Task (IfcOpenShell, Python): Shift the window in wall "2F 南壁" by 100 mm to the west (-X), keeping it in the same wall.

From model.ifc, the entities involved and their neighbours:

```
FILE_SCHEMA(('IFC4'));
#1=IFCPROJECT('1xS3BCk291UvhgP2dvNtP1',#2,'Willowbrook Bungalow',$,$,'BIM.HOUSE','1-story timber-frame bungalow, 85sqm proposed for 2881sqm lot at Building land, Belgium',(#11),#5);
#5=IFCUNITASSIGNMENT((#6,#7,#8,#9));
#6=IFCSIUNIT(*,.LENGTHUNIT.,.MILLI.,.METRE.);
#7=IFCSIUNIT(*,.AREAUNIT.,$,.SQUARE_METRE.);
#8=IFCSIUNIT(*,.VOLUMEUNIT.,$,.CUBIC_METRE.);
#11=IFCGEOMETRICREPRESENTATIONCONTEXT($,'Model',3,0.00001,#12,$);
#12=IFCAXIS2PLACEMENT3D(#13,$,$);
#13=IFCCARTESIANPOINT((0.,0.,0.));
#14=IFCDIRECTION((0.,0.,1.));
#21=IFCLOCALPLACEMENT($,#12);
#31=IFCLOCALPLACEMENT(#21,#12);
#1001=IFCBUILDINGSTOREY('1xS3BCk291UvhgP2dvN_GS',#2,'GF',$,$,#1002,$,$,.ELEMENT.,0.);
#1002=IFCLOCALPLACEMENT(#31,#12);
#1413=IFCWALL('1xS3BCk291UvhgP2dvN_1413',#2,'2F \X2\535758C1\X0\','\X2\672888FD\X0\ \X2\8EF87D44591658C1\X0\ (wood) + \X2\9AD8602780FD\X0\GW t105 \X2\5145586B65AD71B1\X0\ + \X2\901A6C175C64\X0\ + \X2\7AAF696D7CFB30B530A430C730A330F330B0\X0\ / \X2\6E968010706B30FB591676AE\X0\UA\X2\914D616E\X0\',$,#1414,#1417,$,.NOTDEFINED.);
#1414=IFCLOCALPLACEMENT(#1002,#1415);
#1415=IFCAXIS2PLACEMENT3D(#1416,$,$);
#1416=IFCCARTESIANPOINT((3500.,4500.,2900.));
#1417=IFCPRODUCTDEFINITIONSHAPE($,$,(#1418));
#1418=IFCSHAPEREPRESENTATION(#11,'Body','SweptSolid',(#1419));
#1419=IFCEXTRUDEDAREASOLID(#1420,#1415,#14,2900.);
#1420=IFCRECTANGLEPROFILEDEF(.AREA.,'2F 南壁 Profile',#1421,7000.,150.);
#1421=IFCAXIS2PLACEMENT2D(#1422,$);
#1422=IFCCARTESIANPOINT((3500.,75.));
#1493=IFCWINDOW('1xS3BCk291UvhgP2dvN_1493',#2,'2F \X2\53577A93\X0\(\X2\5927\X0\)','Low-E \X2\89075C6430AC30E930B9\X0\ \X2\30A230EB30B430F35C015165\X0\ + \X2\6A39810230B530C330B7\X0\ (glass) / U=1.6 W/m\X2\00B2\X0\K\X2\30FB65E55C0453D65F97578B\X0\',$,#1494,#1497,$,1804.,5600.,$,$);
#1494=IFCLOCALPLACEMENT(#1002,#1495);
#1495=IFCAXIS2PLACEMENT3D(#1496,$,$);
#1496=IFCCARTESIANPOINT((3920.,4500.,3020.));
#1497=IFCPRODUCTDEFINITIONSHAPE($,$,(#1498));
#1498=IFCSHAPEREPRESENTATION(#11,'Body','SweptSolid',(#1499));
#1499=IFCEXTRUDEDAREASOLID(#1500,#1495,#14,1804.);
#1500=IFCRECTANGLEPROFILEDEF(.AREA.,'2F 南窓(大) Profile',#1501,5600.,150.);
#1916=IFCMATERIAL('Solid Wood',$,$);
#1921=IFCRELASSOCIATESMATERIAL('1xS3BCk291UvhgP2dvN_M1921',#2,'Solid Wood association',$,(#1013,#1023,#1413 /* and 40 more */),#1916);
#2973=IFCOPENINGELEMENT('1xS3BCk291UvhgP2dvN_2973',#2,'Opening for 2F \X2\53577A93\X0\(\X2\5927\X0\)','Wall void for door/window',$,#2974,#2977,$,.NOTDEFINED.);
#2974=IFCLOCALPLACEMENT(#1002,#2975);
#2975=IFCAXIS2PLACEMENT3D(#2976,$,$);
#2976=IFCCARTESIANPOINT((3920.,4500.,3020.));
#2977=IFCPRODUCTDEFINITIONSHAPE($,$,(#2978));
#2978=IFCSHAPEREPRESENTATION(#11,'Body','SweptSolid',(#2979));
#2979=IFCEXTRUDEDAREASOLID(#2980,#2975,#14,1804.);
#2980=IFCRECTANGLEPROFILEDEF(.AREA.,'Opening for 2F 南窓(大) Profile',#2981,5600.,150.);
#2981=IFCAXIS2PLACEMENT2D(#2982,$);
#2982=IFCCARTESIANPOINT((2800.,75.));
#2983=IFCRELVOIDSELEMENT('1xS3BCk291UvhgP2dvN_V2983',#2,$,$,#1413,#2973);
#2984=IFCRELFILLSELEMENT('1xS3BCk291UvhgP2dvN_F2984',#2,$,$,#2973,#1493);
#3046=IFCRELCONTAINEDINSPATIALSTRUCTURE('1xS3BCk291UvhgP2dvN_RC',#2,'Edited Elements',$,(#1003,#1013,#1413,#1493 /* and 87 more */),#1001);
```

```python
import ifcopenshell
import ifcopenshell.api.geometry
import ifcopenshell.util.placement
import ifcopenshell.util.unit

model = ifcopenshell.open("model.ifc")
unit_scale = ifcopenshell.util.unit.calculate_unit_scale(model)

window = model.by_guid("1xS3BCk291UvhgP2dvN_1493")
opening = window.FillsVoids[0].RelatingOpeningElement
wall = opening.VoidsElements[0].RelatingBuildingElement

wall_matrix = ifcopenshell.util.placement.get_local_placement(wall.ObjectPlacement)
shift = wall_matrix[:3, 0] * -0.1 / unit_scale
before = ifcopenshell.util.placement.get_local_placement(window.ObjectPlacement)[:3, 3].copy()

# The window is not placed relative to its opening, so move both.
for product in (opening, window):
    matrix = ifcopenshell.util.placement.get_local_placement(product.ObjectPlacement)
    matrix[:3, 3] += shift
    ifcopenshell.api.geometry.edit_object_placement(model, product=product, matrix=matrix, is_si=False)

after = ifcopenshell.util.placement.get_local_placement(window.ObjectPlacement)[:3, 3]
print("window moved by", (after - before).round(3) + 0.0)

model.write("model_updated.ifc")
```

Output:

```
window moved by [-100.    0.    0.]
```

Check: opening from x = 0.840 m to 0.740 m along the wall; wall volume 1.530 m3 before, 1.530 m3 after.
